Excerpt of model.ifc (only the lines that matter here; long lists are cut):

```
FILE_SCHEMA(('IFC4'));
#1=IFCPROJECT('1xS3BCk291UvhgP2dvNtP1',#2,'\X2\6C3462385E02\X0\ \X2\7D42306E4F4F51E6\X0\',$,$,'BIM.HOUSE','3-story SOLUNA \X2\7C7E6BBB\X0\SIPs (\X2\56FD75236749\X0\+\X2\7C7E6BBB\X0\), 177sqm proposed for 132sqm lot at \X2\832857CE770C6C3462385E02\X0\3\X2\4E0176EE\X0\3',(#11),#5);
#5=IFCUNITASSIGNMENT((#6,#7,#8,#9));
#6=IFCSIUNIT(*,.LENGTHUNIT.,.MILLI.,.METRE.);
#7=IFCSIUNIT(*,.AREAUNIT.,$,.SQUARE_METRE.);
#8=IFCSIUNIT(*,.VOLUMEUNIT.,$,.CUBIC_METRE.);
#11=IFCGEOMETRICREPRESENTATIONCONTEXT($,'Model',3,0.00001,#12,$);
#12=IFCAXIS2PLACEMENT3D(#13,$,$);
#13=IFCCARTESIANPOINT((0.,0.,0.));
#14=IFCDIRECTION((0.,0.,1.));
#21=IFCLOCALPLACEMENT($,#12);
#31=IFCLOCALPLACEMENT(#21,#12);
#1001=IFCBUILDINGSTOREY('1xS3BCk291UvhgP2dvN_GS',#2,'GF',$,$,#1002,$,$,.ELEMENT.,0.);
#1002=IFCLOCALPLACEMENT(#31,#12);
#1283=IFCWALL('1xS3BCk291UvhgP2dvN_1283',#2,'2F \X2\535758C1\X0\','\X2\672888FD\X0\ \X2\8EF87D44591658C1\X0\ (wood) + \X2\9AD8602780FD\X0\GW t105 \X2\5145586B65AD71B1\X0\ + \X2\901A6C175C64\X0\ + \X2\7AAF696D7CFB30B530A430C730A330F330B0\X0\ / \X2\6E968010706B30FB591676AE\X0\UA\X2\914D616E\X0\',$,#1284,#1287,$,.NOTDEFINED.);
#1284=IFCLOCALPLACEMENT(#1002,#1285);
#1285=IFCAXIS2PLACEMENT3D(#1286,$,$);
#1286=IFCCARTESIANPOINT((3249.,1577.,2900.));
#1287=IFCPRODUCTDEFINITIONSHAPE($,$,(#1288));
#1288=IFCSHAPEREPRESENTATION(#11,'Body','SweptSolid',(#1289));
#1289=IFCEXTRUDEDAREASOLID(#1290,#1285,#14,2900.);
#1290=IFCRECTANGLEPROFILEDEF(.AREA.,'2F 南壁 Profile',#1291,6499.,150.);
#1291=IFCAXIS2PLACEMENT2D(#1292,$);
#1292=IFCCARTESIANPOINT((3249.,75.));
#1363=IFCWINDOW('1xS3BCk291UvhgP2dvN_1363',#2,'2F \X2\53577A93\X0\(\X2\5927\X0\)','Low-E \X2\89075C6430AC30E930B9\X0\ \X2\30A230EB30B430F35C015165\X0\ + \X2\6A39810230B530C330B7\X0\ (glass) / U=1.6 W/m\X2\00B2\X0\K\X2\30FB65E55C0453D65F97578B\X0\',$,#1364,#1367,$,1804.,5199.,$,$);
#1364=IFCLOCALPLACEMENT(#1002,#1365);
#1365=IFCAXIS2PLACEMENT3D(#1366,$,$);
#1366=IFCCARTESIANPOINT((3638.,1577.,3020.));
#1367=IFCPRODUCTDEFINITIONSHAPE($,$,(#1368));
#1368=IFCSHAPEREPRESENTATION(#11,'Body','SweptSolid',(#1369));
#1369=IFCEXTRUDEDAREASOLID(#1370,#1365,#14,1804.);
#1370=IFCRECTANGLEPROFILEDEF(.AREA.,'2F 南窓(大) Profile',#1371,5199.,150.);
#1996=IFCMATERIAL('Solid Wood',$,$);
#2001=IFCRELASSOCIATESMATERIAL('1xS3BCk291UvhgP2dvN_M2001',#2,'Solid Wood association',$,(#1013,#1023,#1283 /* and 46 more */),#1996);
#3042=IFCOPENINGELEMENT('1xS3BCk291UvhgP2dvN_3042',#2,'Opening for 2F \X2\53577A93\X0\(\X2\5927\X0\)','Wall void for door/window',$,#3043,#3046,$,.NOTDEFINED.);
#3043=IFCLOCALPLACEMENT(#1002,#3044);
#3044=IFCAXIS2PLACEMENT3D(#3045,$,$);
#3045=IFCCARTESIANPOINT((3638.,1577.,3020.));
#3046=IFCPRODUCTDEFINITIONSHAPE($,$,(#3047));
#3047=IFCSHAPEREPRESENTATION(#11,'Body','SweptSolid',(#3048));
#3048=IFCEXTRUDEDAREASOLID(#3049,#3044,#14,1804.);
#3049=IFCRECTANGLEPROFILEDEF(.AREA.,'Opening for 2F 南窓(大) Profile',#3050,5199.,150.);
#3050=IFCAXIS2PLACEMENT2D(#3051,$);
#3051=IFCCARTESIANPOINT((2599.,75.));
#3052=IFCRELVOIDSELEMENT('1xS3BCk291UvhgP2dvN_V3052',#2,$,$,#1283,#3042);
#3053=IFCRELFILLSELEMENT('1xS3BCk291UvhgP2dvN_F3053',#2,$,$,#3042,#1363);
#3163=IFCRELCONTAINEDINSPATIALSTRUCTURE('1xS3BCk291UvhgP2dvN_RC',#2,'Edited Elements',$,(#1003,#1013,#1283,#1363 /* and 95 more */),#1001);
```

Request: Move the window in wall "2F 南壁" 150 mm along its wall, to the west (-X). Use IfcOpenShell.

```python
import ifcopenshell
import ifcopenshell.api.geometry
import ifcopenshell.util.placement
import ifcopenshell.util.unit

model = ifcopenshell.open("model.ifc")
unit_scale = ifcopenshell.util.unit.calculate_unit_scale(model)

window = model.by_guid("1xS3BCk291UvhgP2dvN_1363")
opening = window.FillsVoids[0].RelatingOpeningElement
wall = opening.VoidsElements[0].RelatingBuildingElement

wall_matrix = ifcopenshell.util.placement.get_local_placement(wall.ObjectPlacement)
shift = wall_matrix[:3, 0] * -0.15 / unit_scale
before = ifcopenshell.util.placement.get_local_placement(window.ObjectPlacement)[:3, 3].copy()

# The window is not placed relative to its opening, so move both.
for product in (opening, window):
    matrix = ifcopenshell.util.placement.get_local_placement(product.ObjectPlacement)
    matrix[:3, 3] += shift
    ifcopenshell.api.geometry.edit_object_placement(model, product=product, matrix=matrix, is_si=False)

after = ifcopenshell.util.placement.get_local_placement(window.ObjectPlacement)[:3, 3]
print("window moved by", (after - before).round(3) + 0.0)

model.write("model_updated.ifc")
```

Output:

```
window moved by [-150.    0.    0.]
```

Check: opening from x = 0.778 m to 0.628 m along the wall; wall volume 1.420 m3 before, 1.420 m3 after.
